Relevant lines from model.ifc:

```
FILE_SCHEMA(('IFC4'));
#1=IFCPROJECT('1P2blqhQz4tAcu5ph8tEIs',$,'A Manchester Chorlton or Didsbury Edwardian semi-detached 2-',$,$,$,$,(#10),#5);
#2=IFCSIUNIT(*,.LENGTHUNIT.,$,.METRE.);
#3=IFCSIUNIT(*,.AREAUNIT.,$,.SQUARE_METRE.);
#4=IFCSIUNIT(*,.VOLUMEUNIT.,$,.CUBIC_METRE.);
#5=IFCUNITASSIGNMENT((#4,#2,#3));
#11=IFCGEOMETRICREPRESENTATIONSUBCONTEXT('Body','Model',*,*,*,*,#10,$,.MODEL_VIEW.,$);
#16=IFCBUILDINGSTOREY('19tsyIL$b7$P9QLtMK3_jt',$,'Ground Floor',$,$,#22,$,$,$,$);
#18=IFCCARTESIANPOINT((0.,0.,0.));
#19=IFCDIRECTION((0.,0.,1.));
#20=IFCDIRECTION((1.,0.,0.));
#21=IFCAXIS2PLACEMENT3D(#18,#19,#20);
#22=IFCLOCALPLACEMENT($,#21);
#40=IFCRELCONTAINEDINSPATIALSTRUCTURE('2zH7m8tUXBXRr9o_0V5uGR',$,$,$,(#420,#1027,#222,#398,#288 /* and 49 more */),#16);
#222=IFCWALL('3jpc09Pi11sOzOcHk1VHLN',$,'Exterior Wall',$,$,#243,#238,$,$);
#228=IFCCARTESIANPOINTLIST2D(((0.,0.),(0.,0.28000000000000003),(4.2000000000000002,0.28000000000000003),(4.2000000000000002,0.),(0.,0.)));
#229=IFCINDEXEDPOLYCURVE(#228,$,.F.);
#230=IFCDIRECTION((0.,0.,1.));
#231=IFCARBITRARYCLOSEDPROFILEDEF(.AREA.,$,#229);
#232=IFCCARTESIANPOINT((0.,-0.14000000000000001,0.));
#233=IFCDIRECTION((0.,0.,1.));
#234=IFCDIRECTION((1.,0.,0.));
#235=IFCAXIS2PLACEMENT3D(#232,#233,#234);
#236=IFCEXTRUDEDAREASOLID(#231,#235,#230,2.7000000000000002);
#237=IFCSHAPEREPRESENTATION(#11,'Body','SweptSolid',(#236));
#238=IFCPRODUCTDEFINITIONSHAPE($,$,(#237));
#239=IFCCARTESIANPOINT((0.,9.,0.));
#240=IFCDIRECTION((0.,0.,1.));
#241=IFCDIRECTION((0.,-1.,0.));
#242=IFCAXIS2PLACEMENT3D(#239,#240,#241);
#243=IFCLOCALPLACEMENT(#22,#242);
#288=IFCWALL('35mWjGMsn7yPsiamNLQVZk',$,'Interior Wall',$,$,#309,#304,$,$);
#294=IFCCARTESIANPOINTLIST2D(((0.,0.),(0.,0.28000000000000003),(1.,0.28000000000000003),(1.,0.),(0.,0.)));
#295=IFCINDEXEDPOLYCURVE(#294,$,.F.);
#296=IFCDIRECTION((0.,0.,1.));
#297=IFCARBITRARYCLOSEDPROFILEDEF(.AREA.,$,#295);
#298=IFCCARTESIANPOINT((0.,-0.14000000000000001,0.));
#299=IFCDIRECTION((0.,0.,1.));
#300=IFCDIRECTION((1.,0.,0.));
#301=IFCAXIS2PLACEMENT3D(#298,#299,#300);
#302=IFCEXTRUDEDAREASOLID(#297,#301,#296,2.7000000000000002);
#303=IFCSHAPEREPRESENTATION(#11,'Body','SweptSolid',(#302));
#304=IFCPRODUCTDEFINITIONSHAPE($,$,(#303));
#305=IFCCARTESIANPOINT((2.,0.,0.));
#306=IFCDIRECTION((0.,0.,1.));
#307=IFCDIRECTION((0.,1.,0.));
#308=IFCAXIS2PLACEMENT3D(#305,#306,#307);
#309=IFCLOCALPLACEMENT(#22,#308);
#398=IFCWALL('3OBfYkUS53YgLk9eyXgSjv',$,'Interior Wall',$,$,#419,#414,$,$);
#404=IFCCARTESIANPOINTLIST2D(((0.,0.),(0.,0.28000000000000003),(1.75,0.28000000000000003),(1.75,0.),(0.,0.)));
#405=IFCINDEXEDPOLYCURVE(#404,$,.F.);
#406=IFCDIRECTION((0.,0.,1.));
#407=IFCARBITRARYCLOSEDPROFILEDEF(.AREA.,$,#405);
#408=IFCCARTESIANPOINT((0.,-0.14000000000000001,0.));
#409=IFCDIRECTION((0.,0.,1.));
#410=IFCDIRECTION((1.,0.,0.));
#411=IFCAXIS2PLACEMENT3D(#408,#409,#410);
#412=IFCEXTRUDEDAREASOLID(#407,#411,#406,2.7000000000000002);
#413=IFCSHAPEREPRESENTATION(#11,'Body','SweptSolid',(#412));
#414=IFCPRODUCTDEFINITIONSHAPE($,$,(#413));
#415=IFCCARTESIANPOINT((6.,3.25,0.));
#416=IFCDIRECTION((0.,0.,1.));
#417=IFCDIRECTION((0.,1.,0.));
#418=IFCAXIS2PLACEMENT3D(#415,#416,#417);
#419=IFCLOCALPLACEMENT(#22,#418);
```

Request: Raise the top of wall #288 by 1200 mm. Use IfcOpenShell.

```python
import ifcopenshell
import ifcopenshell.geom
import ifcopenshell.util.representation
import ifcopenshell.util.shape

model = ifcopenshell.open("model.ifc")
settings = ifcopenshell.geom.settings()


def volume(element):
    """Net volume in cubic metres, openings subtracted."""
    shape = ifcopenshell.geom.create_shape(settings, element)
    return ifcopenshell.util.shape.get_volume(shape.geometry)


wall = model.by_id(288)
before = volume(wall)

body = ifcopenshell.util.representation.get_representation(wall, "Model", "Body")
solid = body.Items[0]
old_height = solid.Depth
solid.Depth += 1.2
after = volume(wall)

print(f"height {old_height:g} -> {solid.Depth:g}, volume {before:.3f} -> {after:.3f} m3")

model.write("model_v2.ifc")
```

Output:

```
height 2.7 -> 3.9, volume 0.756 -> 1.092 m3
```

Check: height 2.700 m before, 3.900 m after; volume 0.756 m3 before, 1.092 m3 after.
